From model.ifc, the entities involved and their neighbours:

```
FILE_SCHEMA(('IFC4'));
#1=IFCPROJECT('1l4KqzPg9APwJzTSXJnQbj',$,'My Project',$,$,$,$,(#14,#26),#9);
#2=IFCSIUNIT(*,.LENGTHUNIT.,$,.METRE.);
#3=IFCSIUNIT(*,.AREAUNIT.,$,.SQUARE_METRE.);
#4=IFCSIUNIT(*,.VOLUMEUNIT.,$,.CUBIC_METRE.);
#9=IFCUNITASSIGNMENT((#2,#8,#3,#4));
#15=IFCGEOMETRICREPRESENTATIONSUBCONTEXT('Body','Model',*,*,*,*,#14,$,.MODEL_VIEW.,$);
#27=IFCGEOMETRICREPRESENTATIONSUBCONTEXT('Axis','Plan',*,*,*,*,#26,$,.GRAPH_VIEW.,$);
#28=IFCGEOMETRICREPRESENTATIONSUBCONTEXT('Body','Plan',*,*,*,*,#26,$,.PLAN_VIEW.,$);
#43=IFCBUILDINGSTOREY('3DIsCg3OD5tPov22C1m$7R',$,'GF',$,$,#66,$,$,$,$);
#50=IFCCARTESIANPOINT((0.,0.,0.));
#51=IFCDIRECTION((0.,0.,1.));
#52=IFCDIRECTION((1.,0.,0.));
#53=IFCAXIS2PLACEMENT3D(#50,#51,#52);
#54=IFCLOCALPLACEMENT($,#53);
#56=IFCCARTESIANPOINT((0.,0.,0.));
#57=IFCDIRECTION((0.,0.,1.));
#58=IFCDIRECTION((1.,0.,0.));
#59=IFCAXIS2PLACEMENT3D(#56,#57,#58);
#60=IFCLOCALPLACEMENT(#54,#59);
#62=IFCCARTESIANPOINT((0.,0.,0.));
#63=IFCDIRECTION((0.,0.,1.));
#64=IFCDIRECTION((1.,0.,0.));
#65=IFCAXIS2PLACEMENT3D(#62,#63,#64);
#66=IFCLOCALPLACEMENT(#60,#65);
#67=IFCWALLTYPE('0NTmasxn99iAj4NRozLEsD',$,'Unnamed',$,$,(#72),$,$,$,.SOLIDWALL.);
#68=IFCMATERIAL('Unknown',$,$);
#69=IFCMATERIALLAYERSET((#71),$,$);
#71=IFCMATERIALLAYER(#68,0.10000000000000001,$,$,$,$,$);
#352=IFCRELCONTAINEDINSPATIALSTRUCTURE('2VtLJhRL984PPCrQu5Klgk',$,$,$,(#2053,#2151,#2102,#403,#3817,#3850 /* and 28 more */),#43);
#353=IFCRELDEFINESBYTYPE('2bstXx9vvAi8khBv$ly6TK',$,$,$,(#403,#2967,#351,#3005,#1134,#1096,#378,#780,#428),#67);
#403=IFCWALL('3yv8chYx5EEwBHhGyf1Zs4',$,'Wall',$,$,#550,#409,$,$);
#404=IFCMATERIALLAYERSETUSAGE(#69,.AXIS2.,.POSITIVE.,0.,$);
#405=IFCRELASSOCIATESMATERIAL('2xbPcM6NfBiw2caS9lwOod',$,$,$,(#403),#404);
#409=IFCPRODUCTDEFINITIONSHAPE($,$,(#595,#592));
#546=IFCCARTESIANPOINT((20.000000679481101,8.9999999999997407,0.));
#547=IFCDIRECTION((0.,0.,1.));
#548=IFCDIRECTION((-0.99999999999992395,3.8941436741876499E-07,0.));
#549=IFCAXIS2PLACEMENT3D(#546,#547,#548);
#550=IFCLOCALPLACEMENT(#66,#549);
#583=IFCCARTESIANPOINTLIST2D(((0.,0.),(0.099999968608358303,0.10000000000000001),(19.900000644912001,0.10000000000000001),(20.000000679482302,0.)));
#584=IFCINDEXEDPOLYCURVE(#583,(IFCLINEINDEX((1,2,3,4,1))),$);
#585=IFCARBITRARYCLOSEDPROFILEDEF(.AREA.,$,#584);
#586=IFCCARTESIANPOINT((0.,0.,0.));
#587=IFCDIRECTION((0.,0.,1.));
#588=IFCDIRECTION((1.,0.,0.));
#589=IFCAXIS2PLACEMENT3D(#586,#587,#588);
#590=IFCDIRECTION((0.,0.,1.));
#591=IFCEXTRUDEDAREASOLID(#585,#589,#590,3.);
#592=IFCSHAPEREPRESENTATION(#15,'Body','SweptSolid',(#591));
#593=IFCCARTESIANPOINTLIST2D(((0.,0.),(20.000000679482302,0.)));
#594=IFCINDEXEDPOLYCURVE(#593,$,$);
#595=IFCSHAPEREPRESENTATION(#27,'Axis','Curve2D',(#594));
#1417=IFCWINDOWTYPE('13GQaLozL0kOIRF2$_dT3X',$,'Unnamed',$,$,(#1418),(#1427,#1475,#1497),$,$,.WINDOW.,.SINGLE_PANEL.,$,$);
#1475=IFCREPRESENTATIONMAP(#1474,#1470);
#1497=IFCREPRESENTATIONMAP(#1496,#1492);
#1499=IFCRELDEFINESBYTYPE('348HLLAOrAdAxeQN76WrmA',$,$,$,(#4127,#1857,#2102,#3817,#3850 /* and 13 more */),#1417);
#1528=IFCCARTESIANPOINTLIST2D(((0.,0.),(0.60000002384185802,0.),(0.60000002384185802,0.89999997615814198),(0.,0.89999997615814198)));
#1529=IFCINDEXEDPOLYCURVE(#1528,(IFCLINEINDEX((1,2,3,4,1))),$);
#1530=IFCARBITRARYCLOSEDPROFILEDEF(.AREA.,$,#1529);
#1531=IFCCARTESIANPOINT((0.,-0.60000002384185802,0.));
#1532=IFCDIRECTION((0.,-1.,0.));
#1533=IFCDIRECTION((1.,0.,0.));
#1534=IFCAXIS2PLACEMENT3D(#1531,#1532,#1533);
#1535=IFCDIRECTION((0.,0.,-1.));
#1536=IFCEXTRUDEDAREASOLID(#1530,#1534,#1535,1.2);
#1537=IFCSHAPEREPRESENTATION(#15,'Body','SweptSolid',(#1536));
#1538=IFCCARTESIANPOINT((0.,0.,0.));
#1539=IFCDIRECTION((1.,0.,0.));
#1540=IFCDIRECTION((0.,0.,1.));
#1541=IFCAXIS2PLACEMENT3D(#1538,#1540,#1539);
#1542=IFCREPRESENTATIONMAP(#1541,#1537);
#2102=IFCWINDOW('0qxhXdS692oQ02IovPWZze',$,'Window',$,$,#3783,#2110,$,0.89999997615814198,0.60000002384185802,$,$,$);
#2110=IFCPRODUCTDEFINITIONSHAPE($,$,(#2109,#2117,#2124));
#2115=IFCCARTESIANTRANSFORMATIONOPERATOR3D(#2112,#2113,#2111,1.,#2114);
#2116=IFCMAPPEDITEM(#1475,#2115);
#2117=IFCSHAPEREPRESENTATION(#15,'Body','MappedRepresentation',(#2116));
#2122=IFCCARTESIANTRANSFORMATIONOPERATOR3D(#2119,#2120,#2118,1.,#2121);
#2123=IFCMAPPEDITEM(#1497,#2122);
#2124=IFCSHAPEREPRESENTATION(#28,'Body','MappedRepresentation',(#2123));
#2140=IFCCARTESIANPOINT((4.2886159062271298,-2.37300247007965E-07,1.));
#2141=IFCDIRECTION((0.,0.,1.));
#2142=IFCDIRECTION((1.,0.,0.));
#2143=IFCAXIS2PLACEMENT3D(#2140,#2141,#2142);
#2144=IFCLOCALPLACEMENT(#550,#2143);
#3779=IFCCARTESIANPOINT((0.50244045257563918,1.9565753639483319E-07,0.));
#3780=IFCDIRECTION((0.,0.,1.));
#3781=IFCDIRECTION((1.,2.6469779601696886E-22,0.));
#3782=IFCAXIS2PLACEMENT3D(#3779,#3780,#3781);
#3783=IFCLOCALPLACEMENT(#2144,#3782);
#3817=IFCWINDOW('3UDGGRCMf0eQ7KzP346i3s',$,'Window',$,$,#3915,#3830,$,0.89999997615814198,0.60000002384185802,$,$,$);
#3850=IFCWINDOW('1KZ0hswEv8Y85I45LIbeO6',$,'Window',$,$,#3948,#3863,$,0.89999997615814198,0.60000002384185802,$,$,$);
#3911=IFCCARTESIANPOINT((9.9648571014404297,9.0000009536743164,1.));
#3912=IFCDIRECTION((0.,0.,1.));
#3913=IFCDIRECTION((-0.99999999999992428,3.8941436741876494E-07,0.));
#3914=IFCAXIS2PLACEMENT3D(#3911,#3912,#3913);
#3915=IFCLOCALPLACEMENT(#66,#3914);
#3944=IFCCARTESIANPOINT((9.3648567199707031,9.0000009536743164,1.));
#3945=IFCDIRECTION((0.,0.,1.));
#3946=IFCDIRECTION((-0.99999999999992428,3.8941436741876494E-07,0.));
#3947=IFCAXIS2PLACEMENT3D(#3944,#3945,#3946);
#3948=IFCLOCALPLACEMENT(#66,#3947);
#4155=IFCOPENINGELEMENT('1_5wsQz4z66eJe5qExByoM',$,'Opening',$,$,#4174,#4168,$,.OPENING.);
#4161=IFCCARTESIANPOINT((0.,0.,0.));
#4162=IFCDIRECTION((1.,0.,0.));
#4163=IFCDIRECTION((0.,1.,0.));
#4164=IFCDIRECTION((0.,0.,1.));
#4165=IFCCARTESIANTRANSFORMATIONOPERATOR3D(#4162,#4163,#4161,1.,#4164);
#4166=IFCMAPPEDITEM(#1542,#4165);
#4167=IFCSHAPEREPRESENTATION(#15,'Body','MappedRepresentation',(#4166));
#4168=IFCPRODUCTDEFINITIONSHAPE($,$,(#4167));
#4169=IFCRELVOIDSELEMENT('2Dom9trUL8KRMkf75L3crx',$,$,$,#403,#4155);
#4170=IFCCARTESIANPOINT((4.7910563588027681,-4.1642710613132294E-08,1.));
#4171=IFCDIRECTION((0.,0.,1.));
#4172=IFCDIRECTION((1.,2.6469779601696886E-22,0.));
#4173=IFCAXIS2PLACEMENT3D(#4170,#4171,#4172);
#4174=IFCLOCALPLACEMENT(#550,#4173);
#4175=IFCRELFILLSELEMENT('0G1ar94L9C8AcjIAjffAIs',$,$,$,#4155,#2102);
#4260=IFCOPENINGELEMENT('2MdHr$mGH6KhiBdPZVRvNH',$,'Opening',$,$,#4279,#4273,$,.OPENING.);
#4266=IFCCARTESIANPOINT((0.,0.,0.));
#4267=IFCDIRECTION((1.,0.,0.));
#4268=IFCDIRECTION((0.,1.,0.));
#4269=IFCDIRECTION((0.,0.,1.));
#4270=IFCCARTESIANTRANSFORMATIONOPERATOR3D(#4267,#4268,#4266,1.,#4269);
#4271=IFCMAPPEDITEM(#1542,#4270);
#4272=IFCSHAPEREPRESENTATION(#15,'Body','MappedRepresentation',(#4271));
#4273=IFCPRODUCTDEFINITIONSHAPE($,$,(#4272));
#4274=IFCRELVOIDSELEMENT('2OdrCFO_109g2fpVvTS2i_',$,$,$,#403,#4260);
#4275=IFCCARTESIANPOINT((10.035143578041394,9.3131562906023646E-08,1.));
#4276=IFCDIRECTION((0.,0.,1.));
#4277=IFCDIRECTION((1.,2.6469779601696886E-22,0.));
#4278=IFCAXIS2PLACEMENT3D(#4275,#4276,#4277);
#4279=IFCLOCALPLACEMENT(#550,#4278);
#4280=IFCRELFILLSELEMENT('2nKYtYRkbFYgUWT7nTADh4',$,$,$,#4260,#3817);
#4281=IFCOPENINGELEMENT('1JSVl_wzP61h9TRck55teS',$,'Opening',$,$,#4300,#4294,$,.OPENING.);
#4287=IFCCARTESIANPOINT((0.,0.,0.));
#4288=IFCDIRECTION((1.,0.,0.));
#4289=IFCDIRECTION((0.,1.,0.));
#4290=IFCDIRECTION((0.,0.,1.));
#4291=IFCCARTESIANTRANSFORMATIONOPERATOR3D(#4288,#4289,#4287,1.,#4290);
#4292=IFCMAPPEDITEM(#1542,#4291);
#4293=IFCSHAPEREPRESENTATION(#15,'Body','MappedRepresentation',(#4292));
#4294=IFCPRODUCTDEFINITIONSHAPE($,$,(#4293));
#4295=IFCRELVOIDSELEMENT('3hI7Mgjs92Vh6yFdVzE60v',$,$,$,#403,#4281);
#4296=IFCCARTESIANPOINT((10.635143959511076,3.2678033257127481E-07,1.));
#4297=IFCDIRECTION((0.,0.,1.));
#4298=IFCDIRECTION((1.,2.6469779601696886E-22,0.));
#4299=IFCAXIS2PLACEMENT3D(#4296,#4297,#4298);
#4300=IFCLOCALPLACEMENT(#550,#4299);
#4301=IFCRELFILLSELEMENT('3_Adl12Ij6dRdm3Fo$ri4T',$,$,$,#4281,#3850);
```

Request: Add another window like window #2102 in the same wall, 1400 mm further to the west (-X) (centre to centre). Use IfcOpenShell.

```python
import ifcopenshell
import ifcopenshell.api.feature
import ifcopenshell.api.geometry
import ifcopenshell.api.root
import ifcopenshell.geom
import ifcopenshell.util.element
import ifcopenshell.util.placement
import ifcopenshell.util.shape
import ifcopenshell.util.unit

model = ifcopenshell.open("model.ifc")
unit_scale = ifcopenshell.util.unit.calculate_unit_scale(model)
settings = ifcopenshell.geom.settings()


def volume(element):
    """Net volume in cubic metres, openings subtracted."""
    shape = ifcopenshell.geom.create_shape(settings, element)
    return ifcopenshell.util.shape.get_volume(shape.geometry)


window = model.by_guid("0qxhXdS692oQ02IovPWZze")
opening = window.FillsVoids[0].RelatingOpeningElement
wall = opening.VoidsElements[0].RelatingBuildingElement
before = volume(wall)
shift = ifcopenshell.util.placement.get_local_placement(wall.ObjectPlacement)[:3, 0] * 1.4 / unit_scale

# copy_class copies the void relationship, type, container and properties, but no geometry.
new_opening = ifcopenshell.api.root.copy_class(model, product=opening)
new_opening.Representation = ifcopenshell.util.element.copy_deep(
    model, opening.Representation, exclude=["IfcGeometricRepresentationContext", "IfcRepresentationMap"]
)
new_window = ifcopenshell.api.root.copy_class(model, product=window)
new_window.Representation = ifcopenshell.util.element.copy_deep(
    model, window.Representation, exclude=["IfcGeometricRepresentationContext", "IfcRepresentationMap"]
)
ifcopenshell.api.feature.add_filling(model, opening=new_opening, element=new_window)

for old, new in ((opening, new_opening), (window, new_window)):
    matrix = ifcopenshell.util.placement.get_local_placement(old.ObjectPlacement)
    matrix[:3, 3] += shift
    ifcopenshell.api.geometry.edit_object_placement(model, product=new, matrix=matrix, is_si=False)

after = volume(wall)

print(f"wall volume {before:.3f} -> {after:.3f} m3")

model.write("model_rev.ifc")
```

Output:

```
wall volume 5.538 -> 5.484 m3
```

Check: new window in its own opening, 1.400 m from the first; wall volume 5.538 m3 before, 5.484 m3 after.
